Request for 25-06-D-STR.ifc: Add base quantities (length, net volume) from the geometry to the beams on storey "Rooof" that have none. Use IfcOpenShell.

First a look at what the model holds.

```python
import ifcopenshell
import ifcopenshell.util.element
import ifcopenshell.util.unit

model = ifcopenshell.open("25-06-D-STR.ifc")
print(model.schema)
for unit_type in ("LENGTHUNIT", "AREAUNIT", "VOLUMEUNIT"):
    print(unit_type, ifcopenshell.util.unit.calculate_unit_scale(model, unit_type))
storey = next(s for s in model.by_type("IfcBuildingStorey") if s.Name == "Rooof")
beams = [e for e in ifcopenshell.util.element.get_decomposition(storey) if e.is_a("IfcBeam")]
for e in sorted(beams, key=lambda e: e.id()):
    print(e.id(), e.is_a(), e.Name, list(ifcopenshell.util.element.get_psets(e, qtos_only=True)), sep=" | ")
```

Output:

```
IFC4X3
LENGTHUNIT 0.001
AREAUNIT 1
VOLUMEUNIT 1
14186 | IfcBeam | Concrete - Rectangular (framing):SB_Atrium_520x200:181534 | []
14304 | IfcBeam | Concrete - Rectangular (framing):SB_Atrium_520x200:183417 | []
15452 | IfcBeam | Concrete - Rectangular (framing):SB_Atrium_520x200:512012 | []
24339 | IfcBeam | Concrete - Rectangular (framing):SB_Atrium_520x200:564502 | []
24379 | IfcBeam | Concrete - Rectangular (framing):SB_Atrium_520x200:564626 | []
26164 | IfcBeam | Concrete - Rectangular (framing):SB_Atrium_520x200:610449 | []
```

```python
import ifcopenshell
import ifcopenshell.api.pset
import ifcopenshell.geom
import ifcopenshell.util.element
import ifcopenshell.util.shape
import ifcopenshell.util.unit

model = ifcopenshell.open("25-06-D-STR.ifc")
unit_scale = ifcopenshell.util.unit.calculate_unit_scale(model)
volume_scale = ifcopenshell.util.unit.calculate_unit_scale(model, "VOLUMEUNIT")
settings = ifcopenshell.geom.settings()

storey = next(s for s in model.by_type("IfcBuildingStorey") if s.Name == "Rooof")
beams = [e for e in ifcopenshell.util.element.get_decomposition(storey) if e.is_a("IfcBeam")]

for e in sorted(beams, key=lambda e: e.id()):
    if ifcopenshell.util.element.get_psets(e, qtos_only=True, should_inherit=False):
        continue
    # Geometry comes back in metres, in the element's own axes.
    shape = ifcopenshell.geom.create_shape(settings, e)
    values = {
        "Length": ifcopenshell.util.shape.get_max_xyz(shape.geometry) / unit_scale,
        "NetVolume": ifcopenshell.util.shape.get_volume(shape.geometry) / volume_scale,
    }
    qto = ifcopenshell.api.pset.add_qto(model, product=e, name="Qto_BeamBaseQuantities")
    ifcopenshell.api.pset.edit_qto(model, qto=qto, properties=values)
    print(e.id(), {k: round(v, 3) for k, v in values.items()})

model.write("25-06-D-STR_rev.ifc")
```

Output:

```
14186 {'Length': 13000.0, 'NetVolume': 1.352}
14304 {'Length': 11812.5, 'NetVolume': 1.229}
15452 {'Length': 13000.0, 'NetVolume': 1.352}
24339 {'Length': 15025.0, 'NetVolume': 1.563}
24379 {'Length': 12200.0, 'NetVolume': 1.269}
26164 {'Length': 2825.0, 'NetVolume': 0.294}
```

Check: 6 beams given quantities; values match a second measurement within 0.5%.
